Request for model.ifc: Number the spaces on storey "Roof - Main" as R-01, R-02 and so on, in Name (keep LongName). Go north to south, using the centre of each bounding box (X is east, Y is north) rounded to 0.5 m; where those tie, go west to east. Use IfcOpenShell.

First a look at what the model holds.

```python
import ifcopenshell
import ifcopenshell.util.element
import ifcopenshell.util.placement

model = ifcopenshell.open("model.ifc")
print(model.schema)
storey = next(s for s in model.by_type("IfcBuildingStorey") if s.Name == "Roof - Main")
spaces = [e for e in ifcopenshell.util.element.get_decomposition(storey) if e.is_a("IfcSpace")]
for e in sorted(spaces, key=lambda e: e.id()):
    origin = ifcopenshell.util.placement.get_local_placement(e.ObjectPlacement)[:3, 3]
    print(e.id(), e.Name, e.LongName, origin.round(2) + 0.0, sep=" | ")
```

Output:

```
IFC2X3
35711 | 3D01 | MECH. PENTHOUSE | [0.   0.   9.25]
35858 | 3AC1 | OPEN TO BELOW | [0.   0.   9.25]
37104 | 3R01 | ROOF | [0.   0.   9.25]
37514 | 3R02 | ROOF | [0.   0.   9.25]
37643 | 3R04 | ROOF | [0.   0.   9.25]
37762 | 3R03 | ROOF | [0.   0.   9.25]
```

```python
import ifcopenshell
import ifcopenshell.geom
import ifcopenshell.util.element
import ifcopenshell.util.shape

model = ifcopenshell.open("model.ifc")
settings = ifcopenshell.geom.settings()
settings.set("use-world-coords", True)


def centre(element):
    shape = ifcopenshell.geom.create_shape(settings, element)
    return ifcopenshell.util.shape.get_bbox_centroid(shape.geometry)


storey = next(s for s in model.by_type("IfcBuildingStorey") if s.Name == "Roof - Main")
spaces = [e for e in ifcopenshell.util.element.get_decomposition(storey) if e.is_a("IfcSpace")]

# Insertion points can sit at a corner or the storey origin, so sort by the geometry (in metres).
centres = {e: centre(e) for e in spaces}
spaces.sort(key=lambda e: (-round(centres[e][1] / 0.5), centres[e][0]))

for i, e in enumerate(spaces, start=1):
    number = f"R-{i:02d}"
    e.Name = number
    print(e.id(), number)

model.write("model_v2.ifc")
```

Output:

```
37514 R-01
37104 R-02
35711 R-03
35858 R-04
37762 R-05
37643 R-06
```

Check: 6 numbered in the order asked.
